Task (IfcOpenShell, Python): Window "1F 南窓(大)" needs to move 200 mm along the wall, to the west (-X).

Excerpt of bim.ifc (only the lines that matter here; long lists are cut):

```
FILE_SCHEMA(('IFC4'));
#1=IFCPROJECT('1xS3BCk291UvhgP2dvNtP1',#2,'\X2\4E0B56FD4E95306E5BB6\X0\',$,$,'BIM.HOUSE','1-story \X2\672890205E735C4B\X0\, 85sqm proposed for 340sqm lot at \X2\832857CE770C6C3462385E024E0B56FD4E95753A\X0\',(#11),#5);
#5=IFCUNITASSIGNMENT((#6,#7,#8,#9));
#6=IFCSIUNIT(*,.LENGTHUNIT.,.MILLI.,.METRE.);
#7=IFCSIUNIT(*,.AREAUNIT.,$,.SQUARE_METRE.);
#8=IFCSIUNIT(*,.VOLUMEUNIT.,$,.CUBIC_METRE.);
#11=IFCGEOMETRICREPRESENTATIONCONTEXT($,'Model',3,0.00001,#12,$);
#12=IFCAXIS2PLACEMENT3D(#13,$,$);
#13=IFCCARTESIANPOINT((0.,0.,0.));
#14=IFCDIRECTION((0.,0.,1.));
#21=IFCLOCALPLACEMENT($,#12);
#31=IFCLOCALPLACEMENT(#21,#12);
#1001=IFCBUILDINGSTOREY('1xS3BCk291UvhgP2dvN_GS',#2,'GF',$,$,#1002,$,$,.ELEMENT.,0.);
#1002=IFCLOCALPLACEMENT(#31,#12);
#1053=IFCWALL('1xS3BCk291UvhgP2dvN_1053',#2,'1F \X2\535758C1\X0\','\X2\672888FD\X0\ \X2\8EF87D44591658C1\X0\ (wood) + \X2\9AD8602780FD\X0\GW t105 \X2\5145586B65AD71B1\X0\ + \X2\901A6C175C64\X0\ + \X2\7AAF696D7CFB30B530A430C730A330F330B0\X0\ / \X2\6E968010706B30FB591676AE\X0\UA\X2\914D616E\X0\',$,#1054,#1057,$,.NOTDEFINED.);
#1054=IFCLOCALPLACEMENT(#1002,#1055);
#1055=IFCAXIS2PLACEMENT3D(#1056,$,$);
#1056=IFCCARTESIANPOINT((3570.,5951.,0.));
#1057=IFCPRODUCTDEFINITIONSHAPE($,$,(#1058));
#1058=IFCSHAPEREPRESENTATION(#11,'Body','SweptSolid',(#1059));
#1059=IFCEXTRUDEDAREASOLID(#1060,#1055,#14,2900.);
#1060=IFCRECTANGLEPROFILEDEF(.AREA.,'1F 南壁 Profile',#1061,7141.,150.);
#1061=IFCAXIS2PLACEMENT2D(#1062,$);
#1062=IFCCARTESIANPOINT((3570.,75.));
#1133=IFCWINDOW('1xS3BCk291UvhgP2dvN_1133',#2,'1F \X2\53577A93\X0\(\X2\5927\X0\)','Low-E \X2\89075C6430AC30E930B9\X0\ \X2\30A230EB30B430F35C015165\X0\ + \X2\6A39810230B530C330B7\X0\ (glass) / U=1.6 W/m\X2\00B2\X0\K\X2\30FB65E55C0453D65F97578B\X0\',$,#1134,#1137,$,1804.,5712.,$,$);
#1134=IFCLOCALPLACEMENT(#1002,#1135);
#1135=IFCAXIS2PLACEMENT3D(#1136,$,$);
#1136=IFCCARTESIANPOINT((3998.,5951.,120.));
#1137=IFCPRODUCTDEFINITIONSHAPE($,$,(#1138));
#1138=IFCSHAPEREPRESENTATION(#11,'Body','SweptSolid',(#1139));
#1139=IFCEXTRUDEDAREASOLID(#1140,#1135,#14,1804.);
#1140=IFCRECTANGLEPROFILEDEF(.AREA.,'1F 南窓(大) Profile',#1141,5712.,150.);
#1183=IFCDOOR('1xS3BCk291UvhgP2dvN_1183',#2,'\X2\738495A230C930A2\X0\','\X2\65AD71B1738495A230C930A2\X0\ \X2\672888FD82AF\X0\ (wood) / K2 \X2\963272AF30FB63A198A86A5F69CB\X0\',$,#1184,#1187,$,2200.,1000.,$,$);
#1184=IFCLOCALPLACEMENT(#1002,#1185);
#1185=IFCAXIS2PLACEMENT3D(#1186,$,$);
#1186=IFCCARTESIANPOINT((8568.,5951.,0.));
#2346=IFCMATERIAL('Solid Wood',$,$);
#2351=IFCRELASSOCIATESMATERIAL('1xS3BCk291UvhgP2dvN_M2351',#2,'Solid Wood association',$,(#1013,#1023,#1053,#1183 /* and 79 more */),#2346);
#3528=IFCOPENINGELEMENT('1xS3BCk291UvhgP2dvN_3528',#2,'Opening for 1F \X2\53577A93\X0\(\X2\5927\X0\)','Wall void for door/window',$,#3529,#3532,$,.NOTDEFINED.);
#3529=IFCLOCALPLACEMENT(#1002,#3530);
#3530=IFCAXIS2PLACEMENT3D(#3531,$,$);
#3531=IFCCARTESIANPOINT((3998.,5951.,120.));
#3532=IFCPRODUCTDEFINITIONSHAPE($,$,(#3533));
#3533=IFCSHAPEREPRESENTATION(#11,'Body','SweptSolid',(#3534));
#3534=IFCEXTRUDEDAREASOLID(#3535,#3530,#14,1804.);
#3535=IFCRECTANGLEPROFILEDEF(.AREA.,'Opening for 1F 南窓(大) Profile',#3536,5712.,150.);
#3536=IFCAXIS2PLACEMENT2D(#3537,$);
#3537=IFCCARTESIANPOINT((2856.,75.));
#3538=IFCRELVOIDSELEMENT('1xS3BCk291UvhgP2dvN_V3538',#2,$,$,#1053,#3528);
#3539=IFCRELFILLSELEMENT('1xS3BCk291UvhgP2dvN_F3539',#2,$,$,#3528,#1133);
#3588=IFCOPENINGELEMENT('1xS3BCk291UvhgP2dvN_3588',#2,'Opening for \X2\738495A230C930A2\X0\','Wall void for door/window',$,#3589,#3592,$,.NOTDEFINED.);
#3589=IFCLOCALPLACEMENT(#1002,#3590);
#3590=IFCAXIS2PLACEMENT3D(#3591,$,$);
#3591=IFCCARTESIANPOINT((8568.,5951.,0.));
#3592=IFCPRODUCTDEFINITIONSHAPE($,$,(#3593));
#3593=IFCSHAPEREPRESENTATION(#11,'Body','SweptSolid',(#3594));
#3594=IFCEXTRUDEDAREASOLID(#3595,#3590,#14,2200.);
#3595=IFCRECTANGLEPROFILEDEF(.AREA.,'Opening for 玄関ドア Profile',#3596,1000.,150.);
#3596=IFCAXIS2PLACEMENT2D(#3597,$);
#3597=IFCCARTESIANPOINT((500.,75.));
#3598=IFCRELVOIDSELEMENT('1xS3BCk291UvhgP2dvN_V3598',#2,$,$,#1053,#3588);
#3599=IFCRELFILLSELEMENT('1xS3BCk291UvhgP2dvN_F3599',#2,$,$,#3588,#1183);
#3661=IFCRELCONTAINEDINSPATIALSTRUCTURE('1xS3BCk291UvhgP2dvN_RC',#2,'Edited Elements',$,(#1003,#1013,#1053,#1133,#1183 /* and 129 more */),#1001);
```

```python
import ifcopenshell
import ifcopenshell.api.geometry
import ifcopenshell.util.placement

model = ifcopenshell.open("bim.ifc")

window = model.by_guid("1xS3BCk291UvhgP2dvN_1133")
opening = window.FillsVoids[0].RelatingOpeningElement
wall = opening.VoidsElements[0].RelatingBuildingElement

wall_matrix = ifcopenshell.util.placement.get_local_placement(wall.ObjectPlacement)
shift = wall_matrix[:3, 0] * -200.0
before = ifcopenshell.util.placement.get_local_placement(window.ObjectPlacement)[:3, 3].copy()

# The window is not placed relative to its opening, so move both.
for product in (opening, window):
    matrix = ifcopenshell.util.placement.get_local_placement(product.ObjectPlacement)
    matrix[:3, 3] += shift
    ifcopenshell.api.geometry.edit_object_placement(model, product=product, matrix=matrix, is_si=False)

after = ifcopenshell.util.placement.get_local_placement(window.ObjectPlacement)[:3, 3]
print("window moved by", (after - before).round(3) + 0.0)

model.write("bim_v2.ifc")
```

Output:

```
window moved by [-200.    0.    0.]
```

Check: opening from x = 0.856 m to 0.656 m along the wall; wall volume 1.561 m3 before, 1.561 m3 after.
